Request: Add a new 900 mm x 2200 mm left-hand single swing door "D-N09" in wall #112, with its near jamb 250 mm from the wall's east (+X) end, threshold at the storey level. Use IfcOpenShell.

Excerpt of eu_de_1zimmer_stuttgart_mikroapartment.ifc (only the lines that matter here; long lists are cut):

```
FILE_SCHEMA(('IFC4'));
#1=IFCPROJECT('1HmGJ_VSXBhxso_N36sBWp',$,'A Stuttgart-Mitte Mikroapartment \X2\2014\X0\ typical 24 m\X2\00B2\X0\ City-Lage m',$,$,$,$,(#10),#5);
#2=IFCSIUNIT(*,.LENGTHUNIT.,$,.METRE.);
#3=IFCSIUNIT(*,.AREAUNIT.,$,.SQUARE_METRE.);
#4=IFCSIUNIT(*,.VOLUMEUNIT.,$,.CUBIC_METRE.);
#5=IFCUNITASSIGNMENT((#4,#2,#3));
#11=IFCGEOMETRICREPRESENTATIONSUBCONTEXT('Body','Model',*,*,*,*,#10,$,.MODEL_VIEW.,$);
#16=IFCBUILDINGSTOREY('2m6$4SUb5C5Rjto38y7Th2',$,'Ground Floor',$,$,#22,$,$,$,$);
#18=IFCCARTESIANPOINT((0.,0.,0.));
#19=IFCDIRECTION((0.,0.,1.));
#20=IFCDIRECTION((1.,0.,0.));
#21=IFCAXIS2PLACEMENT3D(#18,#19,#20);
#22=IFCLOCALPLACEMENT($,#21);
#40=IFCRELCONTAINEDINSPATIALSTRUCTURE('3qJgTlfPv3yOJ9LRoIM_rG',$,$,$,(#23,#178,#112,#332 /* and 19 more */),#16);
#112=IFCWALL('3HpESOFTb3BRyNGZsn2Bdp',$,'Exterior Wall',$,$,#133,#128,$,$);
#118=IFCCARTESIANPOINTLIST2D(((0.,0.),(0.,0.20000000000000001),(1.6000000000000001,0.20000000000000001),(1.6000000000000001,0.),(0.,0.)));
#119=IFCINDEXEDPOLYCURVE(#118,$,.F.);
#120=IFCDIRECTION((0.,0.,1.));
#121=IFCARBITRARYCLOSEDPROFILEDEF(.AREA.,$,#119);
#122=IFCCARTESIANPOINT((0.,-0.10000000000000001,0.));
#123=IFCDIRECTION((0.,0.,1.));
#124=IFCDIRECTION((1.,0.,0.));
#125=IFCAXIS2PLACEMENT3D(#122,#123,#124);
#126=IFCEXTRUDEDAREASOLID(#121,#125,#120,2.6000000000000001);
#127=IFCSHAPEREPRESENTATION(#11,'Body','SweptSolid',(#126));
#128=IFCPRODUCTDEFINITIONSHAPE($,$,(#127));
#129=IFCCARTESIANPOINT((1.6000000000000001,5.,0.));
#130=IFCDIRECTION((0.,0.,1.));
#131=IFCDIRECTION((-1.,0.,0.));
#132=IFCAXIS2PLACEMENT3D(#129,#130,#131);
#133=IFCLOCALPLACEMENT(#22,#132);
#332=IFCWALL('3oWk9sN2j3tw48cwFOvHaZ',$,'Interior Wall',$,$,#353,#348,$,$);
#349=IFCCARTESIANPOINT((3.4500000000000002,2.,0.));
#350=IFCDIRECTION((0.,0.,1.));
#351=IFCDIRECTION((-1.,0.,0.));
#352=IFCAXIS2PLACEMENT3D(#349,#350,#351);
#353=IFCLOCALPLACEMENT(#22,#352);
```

```python
import numpy as np
import ifcopenshell
import ifcopenshell.api.feature
import ifcopenshell.api.geometry
import ifcopenshell.api.root
import ifcopenshell.api.spatial
import ifcopenshell.geom
import ifcopenshell.util.element
import ifcopenshell.util.placement
import ifcopenshell.util.representation
import ifcopenshell.util.shape
import ifcopenshell.util.unit

model = ifcopenshell.open("eu_de_1zimmer_stuttgart_mikroapartment.ifc")
unit_scale = ifcopenshell.util.unit.calculate_unit_scale(model)
settings = ifcopenshell.geom.settings()


def volume(element):
    """Net volume in cubic metres, openings subtracted."""
    shape = ifcopenshell.geom.create_shape(settings, element)
    return ifcopenshell.util.shape.get_volume(shape.geometry)


wall = model.by_guid("3HpESOFTb3BRyNGZsn2Bdp")
storey = ifcopenshell.util.element.get_container(wall, ifc_class="IfcBuildingStorey")
context = ifcopenshell.util.representation.get_context(model, "Model", "Body", "MODEL_VIEW")
before = volume(wall)

width, height, from_end, sill = 0.9, 2.2, 0.25, 0.0  # metres

# The wall runs along its own X axis, and the end named is its -X end.
wall_shape = ifcopenshell.geom.create_shape(settings, wall)
x, y, z = ifcopenshell.util.shape.get_vertices(wall_shape.geometry).T
start = x.min() + from_end
face, thickness = float(y.min()), float(y.max() - y.min())
wall_matrix = ifcopenshell.util.placement.get_local_placement(wall.ObjectPlacement)
level = ifcopenshell.util.placement.get_local_placement(storey.ObjectPlacement)[2, 3]


def in_wall(x, y):
    """Placement at x, y metres in the wall's axes, at sill height."""
    matrix = wall_matrix.copy()
    matrix[:, 3] = wall_matrix @ np.array([x / unit_scale, y / unit_scale, 0.0, 1.0])
    matrix[2, 3] = level + sill / unit_scale
    return matrix


# Opening: a box that overshoots both wall faces by 50 mm.
opening = ifcopenshell.api.root.create_entity(model, ifc_class="IfcOpeningElement", predefined_type="OPENING")
box = ifcopenshell.api.geometry.add_wall_representation(
    model, context=context, length=width, height=height, thickness=thickness + 0.1
)
ifcopenshell.api.geometry.assign_representation(model, product=opening, representation=box)
ifcopenshell.api.geometry.edit_object_placement(model, product=opening, matrix=in_wall(start, face - 0.05), is_si=False)
ifcopenshell.api.feature.add_feature(model, feature=opening, element=wall)

door = ifcopenshell.api.root.create_entity(model, ifc_class="IfcDoor", name="D-N09", predefined_type="DOOR")
door.OverallWidth, door.OverallHeight = width / unit_scale, height / unit_scale
door.OperationType = "SINGLE_SWING_LEFT"
body = ifcopenshell.api.geometry.add_door_representation(
    model,
    context=context,
    overall_width=door.OverallWidth,
    overall_height=door.OverallHeight,
    operation_type="SINGLE_SWING_LEFT",
    lining_properties={"LiningDepth": thickness / unit_scale, "ThresholdDepth": thickness / unit_scale},
)
ifcopenshell.api.geometry.assign_representation(model, product=door, representation=body)
ifcopenshell.api.spatial.assign_container(model, products=[door], relating_structure=storey)
ifcopenshell.api.feature.add_filling(model, opening=opening, element=door)

# The lining spans the wall, so the door starts at the wall face.
ifcopenshell.api.geometry.edit_object_placement(model, product=door, matrix=in_wall(start, face), is_si=False)

after = volume(wall)

print(f"wall volume {before:.3f} -> {after:.3f} m3")

model.write("eu_de_1zimmer_stuttgart_mikroapartment_rev.ifc")
```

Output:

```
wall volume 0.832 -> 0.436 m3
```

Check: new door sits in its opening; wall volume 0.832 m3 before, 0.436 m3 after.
